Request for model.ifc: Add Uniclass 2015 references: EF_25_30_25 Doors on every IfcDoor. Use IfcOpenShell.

First a look at what the model holds.

```python
import ifcopenshell

model = ifcopenshell.open("model.ifc")
print(model.schema)
print("classifications:", [c.Name for c in model.by_type("IfcClassification")])
for ifc_class in ("IfcDoor", "IfcRoof", "IfcStair", "IfcWall", "IfcWindow"):
    print(ifc_class, len(model.by_type(ifc_class)))
```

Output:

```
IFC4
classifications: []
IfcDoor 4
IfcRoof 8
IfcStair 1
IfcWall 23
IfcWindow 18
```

```python
import ifcopenshell
import ifcopenshell.api.classification

model = ifcopenshell.open("model.ifc")

system = ifcopenshell.api.classification.add_classification(model, classification="Uniclass 2015")

codes = {
    "IfcDoor": ("EF_25_30_25", "Doors"),
}
for ifc_class, (code, name) in codes.items():
    products = model.by_type(ifc_class)
    ifcopenshell.api.classification.add_reference(
        model, products=products, classification=system, identification=code, name=name
    )
    print(code, len(products))

model.write("model_rev.ifc")
```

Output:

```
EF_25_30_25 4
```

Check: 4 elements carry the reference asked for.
